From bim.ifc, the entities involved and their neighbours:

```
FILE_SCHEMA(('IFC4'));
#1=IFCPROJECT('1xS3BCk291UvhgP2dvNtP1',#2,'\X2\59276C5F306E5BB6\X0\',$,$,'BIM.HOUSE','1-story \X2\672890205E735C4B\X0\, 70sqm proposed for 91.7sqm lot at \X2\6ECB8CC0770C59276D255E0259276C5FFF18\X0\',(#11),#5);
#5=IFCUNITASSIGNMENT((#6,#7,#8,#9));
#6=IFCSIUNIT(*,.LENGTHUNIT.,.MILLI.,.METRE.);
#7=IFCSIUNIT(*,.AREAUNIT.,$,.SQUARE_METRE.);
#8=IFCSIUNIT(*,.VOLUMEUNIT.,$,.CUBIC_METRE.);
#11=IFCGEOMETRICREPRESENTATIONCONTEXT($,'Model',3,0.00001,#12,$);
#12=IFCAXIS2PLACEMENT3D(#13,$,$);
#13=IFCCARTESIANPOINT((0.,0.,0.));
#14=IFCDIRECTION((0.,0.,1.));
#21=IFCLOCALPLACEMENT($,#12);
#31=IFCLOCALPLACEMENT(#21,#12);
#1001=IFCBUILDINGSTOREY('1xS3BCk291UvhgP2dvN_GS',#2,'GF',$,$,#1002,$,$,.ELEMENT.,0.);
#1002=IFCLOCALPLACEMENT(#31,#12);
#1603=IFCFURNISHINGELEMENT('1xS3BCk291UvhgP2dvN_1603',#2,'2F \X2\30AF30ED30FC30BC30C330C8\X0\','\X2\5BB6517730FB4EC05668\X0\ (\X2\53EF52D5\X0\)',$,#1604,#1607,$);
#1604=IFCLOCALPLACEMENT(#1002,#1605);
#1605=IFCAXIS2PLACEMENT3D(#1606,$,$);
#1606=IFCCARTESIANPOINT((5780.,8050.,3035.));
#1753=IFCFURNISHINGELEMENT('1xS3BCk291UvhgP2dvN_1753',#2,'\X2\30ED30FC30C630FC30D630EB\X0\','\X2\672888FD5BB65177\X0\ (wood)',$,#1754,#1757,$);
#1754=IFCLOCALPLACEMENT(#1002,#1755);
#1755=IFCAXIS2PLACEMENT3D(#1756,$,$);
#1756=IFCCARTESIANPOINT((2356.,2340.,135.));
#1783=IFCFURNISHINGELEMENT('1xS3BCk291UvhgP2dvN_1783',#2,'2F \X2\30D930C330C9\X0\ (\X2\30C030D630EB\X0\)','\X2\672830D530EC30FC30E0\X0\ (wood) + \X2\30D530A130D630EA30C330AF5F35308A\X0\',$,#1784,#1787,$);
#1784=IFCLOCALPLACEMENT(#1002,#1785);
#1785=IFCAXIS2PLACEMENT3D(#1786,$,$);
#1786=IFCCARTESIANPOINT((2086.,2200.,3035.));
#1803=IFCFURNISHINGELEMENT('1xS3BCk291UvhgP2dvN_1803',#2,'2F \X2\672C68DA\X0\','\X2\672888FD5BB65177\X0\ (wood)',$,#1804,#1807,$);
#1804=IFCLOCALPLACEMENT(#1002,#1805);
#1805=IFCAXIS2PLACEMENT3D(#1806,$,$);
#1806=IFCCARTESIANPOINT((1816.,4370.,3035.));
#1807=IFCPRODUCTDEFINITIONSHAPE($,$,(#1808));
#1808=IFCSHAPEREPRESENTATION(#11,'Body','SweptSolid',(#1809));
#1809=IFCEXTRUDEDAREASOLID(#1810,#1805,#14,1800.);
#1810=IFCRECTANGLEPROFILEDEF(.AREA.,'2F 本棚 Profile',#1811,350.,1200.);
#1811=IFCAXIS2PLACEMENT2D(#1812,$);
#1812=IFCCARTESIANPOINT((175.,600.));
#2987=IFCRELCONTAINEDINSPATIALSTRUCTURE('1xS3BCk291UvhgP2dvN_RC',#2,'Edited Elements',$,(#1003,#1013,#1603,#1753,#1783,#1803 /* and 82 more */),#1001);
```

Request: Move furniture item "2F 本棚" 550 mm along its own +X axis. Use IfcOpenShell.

```python
import ifcopenshell
import ifcopenshell.api.geometry
import ifcopenshell.util.placement

model = ifcopenshell.open("bim.ifc")

item = model.by_guid("1xS3BCk291UvhgP2dvN_1803")
matrix = ifcopenshell.util.placement.get_local_placement(item.ObjectPlacement)
matrix[:3, 3] += matrix[:3, 0] * 550.0
ifcopenshell.api.geometry.edit_object_placement(model, product=item, matrix=matrix, is_si=False)

print(ifcopenshell.util.placement.get_local_placement(item.ObjectPlacement).round(3) + 0.0)

model.write("bim_rev.ifc")
```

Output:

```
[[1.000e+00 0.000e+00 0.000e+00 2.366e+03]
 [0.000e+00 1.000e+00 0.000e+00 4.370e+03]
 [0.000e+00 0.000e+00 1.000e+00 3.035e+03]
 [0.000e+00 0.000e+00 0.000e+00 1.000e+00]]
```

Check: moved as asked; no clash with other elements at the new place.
